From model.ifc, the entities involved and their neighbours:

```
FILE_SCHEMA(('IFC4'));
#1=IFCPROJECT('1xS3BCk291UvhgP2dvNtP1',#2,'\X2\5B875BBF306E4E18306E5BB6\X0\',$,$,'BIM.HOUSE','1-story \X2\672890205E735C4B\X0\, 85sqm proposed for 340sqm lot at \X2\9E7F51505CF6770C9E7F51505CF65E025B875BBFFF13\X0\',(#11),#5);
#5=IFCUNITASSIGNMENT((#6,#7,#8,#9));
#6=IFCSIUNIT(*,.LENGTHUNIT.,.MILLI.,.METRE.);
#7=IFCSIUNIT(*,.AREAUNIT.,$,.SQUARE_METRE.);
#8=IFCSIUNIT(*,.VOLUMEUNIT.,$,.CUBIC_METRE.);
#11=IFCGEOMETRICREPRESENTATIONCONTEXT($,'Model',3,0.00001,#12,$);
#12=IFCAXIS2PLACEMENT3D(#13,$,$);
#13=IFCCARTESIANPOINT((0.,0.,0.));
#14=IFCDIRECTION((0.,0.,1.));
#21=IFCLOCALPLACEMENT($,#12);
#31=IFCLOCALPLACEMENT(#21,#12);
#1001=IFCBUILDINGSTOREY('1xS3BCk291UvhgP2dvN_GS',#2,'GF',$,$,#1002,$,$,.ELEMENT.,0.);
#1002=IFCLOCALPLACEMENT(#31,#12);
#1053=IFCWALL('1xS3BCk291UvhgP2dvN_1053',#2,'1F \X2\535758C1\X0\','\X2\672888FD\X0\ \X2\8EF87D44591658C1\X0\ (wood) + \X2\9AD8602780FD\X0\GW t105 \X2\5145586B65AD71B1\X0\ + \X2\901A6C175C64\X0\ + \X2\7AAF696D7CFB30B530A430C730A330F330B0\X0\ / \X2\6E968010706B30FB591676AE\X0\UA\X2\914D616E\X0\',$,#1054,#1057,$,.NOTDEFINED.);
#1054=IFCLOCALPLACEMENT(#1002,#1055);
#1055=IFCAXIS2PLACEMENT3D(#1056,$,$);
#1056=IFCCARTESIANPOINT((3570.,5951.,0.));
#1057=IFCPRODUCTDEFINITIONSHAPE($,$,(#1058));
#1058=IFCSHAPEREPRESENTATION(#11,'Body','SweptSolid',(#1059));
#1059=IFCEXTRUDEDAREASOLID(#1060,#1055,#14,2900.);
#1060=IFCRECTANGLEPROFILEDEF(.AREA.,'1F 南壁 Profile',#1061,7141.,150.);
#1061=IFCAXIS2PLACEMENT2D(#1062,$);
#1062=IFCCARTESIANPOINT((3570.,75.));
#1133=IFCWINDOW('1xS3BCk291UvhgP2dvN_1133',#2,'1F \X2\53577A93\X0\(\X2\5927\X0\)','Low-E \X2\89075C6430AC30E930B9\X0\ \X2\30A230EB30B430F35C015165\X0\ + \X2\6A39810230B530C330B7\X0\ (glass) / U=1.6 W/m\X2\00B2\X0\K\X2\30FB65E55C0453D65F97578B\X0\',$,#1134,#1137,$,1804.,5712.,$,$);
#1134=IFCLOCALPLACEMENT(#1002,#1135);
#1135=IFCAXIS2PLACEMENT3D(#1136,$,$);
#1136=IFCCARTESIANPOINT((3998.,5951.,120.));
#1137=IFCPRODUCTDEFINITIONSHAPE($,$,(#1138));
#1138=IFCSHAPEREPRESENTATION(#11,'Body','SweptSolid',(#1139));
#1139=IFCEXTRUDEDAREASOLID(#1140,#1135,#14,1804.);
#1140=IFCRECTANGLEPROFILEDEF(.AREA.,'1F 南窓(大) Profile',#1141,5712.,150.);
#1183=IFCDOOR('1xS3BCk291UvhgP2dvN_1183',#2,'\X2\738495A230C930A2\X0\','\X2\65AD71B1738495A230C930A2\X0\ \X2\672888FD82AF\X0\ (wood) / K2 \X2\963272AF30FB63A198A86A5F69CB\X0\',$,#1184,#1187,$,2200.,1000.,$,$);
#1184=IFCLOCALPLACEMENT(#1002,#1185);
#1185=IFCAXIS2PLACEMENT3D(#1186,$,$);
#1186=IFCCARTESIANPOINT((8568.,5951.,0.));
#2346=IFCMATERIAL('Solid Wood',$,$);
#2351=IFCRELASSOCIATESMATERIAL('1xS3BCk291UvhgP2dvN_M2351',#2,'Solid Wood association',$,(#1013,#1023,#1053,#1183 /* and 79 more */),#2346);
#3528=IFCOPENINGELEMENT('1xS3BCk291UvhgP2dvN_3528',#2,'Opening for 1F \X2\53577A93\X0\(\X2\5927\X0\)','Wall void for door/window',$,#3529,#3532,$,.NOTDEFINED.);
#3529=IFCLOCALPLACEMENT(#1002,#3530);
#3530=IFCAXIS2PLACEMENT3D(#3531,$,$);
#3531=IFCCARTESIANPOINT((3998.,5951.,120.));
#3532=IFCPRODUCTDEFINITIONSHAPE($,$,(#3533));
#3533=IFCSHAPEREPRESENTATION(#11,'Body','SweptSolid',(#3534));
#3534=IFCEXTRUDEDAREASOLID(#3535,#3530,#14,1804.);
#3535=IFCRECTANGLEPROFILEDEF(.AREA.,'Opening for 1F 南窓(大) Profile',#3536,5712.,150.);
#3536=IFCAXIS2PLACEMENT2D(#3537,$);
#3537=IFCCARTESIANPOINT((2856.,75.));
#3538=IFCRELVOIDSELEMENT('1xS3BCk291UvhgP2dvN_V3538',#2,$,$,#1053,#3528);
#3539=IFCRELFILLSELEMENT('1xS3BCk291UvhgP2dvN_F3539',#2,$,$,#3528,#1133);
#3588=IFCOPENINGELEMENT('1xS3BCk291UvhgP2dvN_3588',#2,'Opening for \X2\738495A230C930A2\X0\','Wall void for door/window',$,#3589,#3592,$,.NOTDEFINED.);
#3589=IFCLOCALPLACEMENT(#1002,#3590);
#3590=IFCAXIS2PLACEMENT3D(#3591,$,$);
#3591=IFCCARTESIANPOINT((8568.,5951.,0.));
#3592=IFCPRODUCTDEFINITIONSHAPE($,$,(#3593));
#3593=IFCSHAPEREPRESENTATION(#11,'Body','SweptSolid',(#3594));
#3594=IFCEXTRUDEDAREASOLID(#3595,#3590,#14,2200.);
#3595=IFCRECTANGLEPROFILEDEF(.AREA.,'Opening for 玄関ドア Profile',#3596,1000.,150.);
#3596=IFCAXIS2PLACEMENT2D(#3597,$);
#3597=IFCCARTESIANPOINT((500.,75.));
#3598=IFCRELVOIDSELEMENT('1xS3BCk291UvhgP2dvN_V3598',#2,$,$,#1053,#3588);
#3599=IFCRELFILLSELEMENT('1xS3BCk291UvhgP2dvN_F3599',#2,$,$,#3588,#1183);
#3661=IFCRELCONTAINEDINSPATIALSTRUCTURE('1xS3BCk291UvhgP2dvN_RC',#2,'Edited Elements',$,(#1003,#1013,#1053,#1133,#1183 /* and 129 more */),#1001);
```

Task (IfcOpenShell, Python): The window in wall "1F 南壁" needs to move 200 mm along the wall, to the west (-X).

```python
import ifcopenshell
import ifcopenshell.api.geometry
import ifcopenshell.util.placement

model = ifcopenshell.open("model.ifc")

window = model.by_guid("1xS3BCk291UvhgP2dvN_1133")
opening = window.FillsVoids[0].RelatingOpeningElement
wall = opening.VoidsElements[0].RelatingBuildingElement

wall_matrix = ifcopenshell.util.placement.get_local_placement(wall.ObjectPlacement)
shift = wall_matrix[:3, 0] * -200.0
before = ifcopenshell.util.placement.get_local_placement(window.ObjectPlacement)[:3, 3].copy()

# The window is not placed relative to its opening, so move both.
for product in (opening, window):
    matrix = ifcopenshell.util.placement.get_local_placement(product.ObjectPlacement)
    matrix[:3, 3] += shift
    ifcopenshell.api.geometry.edit_object_placement(model, product=product, matrix=matrix, is_si=False)

after = ifcopenshell.util.placement.get_local_placement(window.ObjectPlacement)[:3, 3]
print("window moved by", (after - before).round(3) + 0.0)

model.write("model_edited.ifc")
```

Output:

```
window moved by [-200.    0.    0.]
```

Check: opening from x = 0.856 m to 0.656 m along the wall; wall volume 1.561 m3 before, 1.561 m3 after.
